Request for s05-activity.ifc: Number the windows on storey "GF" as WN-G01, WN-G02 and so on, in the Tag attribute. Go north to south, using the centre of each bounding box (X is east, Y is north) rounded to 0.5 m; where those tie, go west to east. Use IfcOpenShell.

First a look at what the model holds.

```python
import ifcopenshell
import ifcopenshell.util.element
import ifcopenshell.util.placement

model = ifcopenshell.open("s05-activity.ifc")
print(model.schema)
storey = next(s for s in model.by_type("IfcBuildingStorey") if s.Name == "GF")
windows = [e for e in ifcopenshell.util.element.get_decomposition(storey) if e.is_a("IfcWindow")]
for e in sorted(windows, key=lambda e: e.id()):
    origin = ifcopenshell.util.placement.get_local_placement(e.ObjectPlacement)[:3, 3]
    print(e.id(), e.Tag, e.Name, origin.round(2) + 0.0, sep=" | ")
```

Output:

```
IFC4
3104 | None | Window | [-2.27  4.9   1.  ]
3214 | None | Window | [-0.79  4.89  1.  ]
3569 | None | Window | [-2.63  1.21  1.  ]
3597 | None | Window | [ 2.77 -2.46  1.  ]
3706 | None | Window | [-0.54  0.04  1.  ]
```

```python
import ifcopenshell
import ifcopenshell.geom
import ifcopenshell.util.element
import ifcopenshell.util.shape

model = ifcopenshell.open("s05-activity.ifc")
settings = ifcopenshell.geom.settings()
settings.set("use-world-coords", True)


def centre(element):
    shape = ifcopenshell.geom.create_shape(settings, element)
    return ifcopenshell.util.shape.get_bbox_centroid(shape.geometry)


storey = next(s for s in model.by_type("IfcBuildingStorey") if s.Name == "GF")
windows = [e for e in ifcopenshell.util.element.get_decomposition(storey) if e.is_a("IfcWindow")]

# Insertion points can sit at a corner or the storey origin, so sort by the geometry (in metres).
centres = {e: centre(e) for e in windows}
windows.sort(key=lambda e: (-round(centres[e][1] / 0.5), centres[e][0]))

for i, e in enumerate(windows, start=1):
    number = f"WN-G{i:02d}"
    e.Tag = number
    print(e.id(), number)

model.write("s05-activity_v2.ifc")
```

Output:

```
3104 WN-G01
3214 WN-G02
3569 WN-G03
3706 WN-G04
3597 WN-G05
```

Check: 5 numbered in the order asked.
